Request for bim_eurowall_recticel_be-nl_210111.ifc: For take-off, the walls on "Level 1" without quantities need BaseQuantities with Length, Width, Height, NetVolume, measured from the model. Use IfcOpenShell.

First a look at what the model holds.

```python
import ifcopenshell
import ifcopenshell.util.element
import ifcopenshell.util.unit

model = ifcopenshell.open("bim_eurowall_recticel_be-nl_210111.ifc")
print(model.schema)
for unit_type in ("LENGTHUNIT", "AREAUNIT", "VOLUMEUNIT"):
    print(unit_type, ifcopenshell.util.unit.calculate_unit_scale(model, unit_type))
storey = next(s for s in model.by_type("IfcBuildingStorey") if s.Name == "Level 1")
walls = [e for e in ifcopenshell.util.element.get_decomposition(storey) if e.is_a("IfcWall")]
for e in sorted(walls, key=lambda e: e.id()):
    print(e.id(), e.is_a(), e.Name, list(ifcopenshell.util.element.get_psets(e, qtos_only=True)), sep=" | ")
```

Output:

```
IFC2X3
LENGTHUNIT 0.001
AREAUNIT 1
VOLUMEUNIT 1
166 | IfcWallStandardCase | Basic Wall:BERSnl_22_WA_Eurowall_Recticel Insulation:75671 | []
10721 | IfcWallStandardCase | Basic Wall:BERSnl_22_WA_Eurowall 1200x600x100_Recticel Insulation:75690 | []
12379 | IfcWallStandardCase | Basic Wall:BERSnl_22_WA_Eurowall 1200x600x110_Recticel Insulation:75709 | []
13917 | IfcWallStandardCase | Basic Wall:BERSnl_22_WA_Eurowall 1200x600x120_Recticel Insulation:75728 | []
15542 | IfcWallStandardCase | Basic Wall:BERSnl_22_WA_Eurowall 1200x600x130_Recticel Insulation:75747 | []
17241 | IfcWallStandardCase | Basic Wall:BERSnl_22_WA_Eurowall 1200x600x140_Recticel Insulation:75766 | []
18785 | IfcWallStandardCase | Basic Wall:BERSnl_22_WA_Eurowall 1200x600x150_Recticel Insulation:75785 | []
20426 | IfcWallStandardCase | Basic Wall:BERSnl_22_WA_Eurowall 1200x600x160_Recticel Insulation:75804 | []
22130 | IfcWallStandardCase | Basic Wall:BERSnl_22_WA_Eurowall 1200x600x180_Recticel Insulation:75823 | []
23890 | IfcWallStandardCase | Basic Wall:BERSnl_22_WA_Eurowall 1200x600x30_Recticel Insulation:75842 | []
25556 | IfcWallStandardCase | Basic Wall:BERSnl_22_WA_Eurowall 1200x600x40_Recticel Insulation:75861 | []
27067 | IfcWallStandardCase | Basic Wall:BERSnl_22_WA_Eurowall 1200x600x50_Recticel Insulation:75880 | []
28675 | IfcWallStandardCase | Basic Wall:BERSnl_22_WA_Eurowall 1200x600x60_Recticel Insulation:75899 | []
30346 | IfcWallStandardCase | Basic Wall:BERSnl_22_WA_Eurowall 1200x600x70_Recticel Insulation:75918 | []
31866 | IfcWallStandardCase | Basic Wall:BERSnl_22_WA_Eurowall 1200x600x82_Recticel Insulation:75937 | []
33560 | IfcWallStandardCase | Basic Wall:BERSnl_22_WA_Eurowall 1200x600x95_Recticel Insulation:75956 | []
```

```python
import ifcopenshell
import ifcopenshell.api.pset
import ifcopenshell.geom
import ifcopenshell.util.element
import ifcopenshell.util.shape
import ifcopenshell.util.unit

model = ifcopenshell.open("bim_eurowall_recticel_be-nl_210111.ifc")
unit_scale = ifcopenshell.util.unit.calculate_unit_scale(model)
volume_scale = ifcopenshell.util.unit.calculate_unit_scale(model, "VOLUMEUNIT")
settings = ifcopenshell.geom.settings()

storey = next(s for s in model.by_type("IfcBuildingStorey") if s.Name == "Level 1")
walls = [e for e in ifcopenshell.util.element.get_decomposition(storey) if e.is_a("IfcWall")]

for e in sorted(walls, key=lambda e: e.id()):
    if ifcopenshell.util.element.get_psets(e, qtos_only=True, should_inherit=False):
        continue
    # Geometry comes back in metres, in the element's own axes.
    shape = ifcopenshell.geom.create_shape(settings, e)
    values = {
        "Length": ifcopenshell.util.shape.get_x(shape.geometry) / unit_scale,
        "Width": ifcopenshell.util.shape.get_y(shape.geometry) / unit_scale,
        "Height": ifcopenshell.util.shape.get_z(shape.geometry) / unit_scale,
        "NetVolume": ifcopenshell.util.shape.get_volume(shape.geometry) / volume_scale,
    }
    qto = ifcopenshell.api.pset.add_qto(model, product=e, name="BaseQuantities")
    ifcopenshell.api.pset.edit_qto(model, qto=qto, properties=values)
    print(e.id(), {k: round(v, 3) for k, v in values.items()})

model.write("bim_eurowall_recticel_be-nl_210111_v2.ifc")
```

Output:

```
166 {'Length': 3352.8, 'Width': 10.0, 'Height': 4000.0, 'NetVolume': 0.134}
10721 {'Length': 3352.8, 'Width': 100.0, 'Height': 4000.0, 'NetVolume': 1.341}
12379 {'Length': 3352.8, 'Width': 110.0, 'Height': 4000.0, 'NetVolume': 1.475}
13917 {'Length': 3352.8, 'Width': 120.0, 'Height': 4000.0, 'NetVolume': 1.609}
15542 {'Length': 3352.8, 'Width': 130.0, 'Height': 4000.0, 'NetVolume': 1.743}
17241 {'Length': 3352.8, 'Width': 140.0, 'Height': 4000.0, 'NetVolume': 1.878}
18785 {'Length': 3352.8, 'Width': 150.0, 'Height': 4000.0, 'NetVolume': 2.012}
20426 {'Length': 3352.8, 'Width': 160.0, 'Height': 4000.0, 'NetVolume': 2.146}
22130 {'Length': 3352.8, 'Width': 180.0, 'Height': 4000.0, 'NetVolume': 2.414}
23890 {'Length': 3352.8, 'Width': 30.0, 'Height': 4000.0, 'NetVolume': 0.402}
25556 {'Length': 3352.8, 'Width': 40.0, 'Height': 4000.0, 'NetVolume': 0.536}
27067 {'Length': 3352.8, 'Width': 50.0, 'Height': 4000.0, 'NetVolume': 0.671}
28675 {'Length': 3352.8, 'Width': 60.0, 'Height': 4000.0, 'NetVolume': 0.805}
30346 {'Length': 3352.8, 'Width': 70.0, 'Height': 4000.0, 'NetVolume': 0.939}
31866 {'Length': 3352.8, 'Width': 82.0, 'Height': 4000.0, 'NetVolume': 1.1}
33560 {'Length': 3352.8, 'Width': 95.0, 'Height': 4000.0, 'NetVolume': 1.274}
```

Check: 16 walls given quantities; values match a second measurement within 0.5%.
